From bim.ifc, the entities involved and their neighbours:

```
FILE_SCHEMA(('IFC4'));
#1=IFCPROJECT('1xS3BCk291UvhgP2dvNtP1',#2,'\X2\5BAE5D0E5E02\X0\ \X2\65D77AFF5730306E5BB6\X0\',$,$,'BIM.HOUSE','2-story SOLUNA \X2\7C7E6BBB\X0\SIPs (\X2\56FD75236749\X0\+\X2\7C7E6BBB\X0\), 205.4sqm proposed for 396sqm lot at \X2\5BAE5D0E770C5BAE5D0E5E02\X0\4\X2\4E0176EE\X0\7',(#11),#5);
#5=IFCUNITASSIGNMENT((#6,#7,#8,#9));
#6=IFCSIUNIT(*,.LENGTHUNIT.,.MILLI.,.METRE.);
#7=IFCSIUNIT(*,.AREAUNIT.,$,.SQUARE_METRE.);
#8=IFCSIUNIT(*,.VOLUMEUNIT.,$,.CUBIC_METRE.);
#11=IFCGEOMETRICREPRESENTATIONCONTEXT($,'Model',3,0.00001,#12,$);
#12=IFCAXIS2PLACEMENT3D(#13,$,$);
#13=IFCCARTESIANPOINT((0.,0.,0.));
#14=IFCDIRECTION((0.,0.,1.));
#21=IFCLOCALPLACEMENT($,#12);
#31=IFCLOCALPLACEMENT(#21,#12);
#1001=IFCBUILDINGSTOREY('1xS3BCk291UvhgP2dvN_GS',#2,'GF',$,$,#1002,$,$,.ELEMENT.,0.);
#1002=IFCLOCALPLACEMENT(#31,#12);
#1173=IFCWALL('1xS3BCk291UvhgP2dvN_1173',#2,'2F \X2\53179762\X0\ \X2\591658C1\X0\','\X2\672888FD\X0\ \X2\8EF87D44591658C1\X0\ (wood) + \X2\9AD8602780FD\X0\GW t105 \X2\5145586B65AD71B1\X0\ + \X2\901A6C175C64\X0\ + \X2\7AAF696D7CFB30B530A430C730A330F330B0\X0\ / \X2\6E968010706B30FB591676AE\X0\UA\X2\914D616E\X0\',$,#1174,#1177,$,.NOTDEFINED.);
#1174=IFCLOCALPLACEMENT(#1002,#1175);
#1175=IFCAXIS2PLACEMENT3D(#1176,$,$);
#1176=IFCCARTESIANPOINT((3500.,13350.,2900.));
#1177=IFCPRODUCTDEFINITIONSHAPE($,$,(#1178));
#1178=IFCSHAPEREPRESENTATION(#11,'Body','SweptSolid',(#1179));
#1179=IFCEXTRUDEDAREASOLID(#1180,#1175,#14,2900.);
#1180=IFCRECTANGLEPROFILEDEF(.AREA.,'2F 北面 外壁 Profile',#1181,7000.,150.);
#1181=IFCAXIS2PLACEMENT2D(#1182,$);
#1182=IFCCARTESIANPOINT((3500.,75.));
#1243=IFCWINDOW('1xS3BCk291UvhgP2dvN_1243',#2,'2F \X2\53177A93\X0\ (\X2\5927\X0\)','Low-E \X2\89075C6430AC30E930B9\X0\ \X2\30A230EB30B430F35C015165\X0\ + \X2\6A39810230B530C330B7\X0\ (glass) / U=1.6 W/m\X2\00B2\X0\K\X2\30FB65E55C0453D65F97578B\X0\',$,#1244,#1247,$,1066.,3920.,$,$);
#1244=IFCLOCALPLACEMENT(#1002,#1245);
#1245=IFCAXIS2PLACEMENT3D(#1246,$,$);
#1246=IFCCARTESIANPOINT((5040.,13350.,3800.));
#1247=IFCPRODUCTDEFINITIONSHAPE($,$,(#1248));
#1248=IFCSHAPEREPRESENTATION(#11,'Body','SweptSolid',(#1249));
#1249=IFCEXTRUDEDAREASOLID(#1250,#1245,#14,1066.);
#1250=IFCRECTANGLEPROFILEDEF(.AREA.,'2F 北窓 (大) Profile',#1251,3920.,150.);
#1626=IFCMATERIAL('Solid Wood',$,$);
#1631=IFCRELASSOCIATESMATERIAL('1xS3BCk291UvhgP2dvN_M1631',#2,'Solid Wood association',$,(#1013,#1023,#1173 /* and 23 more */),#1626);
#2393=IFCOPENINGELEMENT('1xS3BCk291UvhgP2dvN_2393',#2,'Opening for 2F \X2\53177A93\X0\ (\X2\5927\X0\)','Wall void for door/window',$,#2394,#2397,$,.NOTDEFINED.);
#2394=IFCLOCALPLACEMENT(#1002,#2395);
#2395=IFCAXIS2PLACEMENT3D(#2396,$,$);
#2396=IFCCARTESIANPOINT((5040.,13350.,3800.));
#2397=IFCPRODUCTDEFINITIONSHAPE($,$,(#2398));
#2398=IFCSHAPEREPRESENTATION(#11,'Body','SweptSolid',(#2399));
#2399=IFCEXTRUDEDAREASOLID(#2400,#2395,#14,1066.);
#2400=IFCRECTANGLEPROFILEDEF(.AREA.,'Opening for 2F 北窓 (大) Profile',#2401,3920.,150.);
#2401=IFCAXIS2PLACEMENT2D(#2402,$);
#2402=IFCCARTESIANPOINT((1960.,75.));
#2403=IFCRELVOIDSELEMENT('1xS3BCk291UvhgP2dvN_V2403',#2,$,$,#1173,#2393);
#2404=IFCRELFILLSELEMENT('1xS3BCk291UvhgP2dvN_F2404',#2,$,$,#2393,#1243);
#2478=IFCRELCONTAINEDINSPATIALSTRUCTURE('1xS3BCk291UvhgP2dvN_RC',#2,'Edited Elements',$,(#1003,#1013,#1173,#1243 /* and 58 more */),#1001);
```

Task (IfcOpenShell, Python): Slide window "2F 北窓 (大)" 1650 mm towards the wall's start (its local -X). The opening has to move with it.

```python
import ifcopenshell
import ifcopenshell.api.geometry
import ifcopenshell.util.placement
import ifcopenshell.util.unit

model = ifcopenshell.open("bim.ifc")
unit_scale = ifcopenshell.util.unit.calculate_unit_scale(model)

window = model.by_guid("1xS3BCk291UvhgP2dvN_1243")
opening = window.FillsVoids[0].RelatingOpeningElement
wall = opening.VoidsElements[0].RelatingBuildingElement

wall_matrix = ifcopenshell.util.placement.get_local_placement(wall.ObjectPlacement)
shift = wall_matrix[:3, 0] * -1.65 / unit_scale
before = ifcopenshell.util.placement.get_local_placement(window.ObjectPlacement)[:3, 3].copy()

# The window is not placed relative to its opening, so move both.
for product in (opening, window):
    matrix = ifcopenshell.util.placement.get_local_placement(product.ObjectPlacement)
    matrix[:3, 3] += shift
    ifcopenshell.api.geometry.edit_object_placement(model, product=product, matrix=matrix, is_si=False)

after = ifcopenshell.util.placement.get_local_placement(window.ObjectPlacement)[:3, 3]
print("window moved by", (after - before).round(3) + 0.0)

model.write("bim_updated.ifc")
```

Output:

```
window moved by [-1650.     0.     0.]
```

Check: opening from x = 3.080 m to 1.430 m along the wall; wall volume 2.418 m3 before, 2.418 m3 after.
